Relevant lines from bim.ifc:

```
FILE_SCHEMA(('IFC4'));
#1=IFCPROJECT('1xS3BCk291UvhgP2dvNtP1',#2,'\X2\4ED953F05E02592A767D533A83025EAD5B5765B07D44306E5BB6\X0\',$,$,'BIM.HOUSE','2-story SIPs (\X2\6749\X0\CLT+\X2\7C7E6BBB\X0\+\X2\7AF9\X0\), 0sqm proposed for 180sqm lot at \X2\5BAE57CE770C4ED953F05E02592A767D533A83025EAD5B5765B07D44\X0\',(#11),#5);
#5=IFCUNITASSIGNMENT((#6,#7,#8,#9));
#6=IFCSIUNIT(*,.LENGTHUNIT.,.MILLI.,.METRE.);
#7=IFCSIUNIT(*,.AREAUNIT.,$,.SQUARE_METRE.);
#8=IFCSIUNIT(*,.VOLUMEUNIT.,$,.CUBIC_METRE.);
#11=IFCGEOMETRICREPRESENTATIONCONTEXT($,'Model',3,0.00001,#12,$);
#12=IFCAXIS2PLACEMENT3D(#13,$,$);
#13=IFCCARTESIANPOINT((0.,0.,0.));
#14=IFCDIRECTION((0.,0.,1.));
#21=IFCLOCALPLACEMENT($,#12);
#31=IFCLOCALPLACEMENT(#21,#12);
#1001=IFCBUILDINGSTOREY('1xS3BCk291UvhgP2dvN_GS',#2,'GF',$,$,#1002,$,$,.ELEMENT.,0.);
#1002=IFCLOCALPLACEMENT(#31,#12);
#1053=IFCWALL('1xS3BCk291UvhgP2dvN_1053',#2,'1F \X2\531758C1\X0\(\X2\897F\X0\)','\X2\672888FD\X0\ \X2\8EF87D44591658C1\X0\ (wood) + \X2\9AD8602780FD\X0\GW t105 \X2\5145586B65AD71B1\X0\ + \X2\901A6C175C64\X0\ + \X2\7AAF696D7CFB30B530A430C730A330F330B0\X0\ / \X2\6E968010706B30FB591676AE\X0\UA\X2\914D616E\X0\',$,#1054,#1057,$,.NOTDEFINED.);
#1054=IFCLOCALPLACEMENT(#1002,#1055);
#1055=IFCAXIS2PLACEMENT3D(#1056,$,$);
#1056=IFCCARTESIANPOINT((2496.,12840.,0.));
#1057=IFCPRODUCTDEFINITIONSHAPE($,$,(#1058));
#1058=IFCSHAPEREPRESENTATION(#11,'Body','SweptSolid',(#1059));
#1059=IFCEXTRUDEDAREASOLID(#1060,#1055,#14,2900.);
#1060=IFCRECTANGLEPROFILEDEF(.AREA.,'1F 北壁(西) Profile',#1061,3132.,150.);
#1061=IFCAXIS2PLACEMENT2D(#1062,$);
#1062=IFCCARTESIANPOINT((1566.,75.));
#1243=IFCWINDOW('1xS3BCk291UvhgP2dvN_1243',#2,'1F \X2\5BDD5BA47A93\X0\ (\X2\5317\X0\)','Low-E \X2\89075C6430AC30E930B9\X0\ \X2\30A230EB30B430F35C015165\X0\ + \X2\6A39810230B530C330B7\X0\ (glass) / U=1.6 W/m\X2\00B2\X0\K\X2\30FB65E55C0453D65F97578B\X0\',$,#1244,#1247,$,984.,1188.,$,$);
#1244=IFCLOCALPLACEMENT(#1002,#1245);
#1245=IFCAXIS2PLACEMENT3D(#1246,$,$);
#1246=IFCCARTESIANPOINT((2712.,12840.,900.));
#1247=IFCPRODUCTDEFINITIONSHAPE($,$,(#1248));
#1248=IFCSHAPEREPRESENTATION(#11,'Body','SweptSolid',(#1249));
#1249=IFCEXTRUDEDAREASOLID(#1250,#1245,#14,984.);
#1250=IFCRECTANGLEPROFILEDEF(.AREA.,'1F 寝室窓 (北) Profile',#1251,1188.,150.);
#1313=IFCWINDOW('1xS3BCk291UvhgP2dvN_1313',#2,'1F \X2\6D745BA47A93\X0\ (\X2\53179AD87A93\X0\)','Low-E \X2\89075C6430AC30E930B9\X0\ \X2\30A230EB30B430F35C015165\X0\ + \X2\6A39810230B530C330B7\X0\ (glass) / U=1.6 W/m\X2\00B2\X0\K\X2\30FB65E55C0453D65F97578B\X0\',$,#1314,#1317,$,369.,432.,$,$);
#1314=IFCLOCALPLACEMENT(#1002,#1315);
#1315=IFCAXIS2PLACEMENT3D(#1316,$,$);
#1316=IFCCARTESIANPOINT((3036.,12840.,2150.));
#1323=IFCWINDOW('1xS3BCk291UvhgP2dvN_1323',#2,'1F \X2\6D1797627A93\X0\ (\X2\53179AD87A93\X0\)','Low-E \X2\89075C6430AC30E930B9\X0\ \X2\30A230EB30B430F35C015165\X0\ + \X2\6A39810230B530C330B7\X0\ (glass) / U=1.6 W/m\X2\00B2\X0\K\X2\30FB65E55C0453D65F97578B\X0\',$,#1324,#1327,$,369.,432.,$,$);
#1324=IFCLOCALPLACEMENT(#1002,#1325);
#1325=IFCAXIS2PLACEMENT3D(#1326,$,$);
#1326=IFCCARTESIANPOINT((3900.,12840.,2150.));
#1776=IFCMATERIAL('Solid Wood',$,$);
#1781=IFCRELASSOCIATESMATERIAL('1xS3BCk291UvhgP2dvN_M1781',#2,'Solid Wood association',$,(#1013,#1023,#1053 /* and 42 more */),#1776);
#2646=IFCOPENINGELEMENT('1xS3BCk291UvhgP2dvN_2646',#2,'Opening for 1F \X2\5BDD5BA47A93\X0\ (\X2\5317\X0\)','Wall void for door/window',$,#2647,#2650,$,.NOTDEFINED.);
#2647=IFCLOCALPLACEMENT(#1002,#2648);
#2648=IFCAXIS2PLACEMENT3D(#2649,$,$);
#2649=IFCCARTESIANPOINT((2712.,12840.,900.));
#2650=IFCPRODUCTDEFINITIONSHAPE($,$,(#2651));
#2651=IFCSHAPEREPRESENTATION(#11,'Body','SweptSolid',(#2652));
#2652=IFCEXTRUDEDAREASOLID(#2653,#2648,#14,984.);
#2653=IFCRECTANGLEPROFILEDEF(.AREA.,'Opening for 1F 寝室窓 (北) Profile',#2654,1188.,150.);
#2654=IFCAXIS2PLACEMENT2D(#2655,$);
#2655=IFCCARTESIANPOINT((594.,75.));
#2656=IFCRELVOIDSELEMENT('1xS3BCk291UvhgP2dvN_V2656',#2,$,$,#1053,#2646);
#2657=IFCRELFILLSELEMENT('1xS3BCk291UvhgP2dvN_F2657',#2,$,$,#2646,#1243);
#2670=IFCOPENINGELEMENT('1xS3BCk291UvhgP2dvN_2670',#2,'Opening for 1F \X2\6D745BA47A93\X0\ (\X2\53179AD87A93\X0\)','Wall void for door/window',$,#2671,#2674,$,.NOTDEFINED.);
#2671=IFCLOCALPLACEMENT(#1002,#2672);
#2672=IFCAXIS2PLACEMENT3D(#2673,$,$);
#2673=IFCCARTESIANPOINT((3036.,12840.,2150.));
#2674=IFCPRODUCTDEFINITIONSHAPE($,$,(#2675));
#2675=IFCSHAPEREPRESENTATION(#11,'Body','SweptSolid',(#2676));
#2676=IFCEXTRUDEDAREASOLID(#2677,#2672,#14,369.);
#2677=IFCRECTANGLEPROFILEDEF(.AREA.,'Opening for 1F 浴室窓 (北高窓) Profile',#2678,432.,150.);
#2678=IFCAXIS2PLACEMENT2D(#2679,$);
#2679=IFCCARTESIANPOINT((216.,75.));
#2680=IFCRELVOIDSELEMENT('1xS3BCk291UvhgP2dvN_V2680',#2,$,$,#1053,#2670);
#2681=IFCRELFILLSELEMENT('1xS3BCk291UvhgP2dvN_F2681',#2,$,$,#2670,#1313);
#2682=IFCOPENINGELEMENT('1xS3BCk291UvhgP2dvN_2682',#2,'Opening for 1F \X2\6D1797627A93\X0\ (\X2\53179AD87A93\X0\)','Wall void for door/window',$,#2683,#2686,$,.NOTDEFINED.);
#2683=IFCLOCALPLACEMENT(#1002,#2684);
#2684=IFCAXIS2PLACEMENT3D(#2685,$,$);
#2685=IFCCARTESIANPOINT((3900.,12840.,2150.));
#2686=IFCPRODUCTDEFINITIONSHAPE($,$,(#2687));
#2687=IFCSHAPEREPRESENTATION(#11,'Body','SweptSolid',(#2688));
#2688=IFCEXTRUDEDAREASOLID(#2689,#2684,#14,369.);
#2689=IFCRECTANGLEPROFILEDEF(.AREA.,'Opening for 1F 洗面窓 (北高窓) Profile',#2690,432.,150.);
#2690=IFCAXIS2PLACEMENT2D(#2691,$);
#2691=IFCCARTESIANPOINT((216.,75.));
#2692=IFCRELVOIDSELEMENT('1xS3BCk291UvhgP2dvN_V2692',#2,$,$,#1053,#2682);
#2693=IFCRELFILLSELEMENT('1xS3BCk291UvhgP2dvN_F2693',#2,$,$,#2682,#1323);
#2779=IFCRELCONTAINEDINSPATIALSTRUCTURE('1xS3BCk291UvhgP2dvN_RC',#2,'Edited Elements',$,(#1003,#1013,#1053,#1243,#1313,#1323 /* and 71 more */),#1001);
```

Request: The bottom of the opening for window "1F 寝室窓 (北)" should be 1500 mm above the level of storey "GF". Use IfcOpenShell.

```python
import numpy as np
import ifcopenshell
import ifcopenshell.api.geometry
import ifcopenshell.geom
import ifcopenshell.util.element
import ifcopenshell.util.placement
import ifcopenshell.util.shape
import ifcopenshell.util.unit

model = ifcopenshell.open("bim.ifc")
unit_scale = ifcopenshell.util.unit.calculate_unit_scale(model)

window = model.by_id(1243)
opening = window.FillsVoids[0].RelatingOpeningElement
storey = ifcopenshell.util.element.get_container(window, ifc_class="IfcBuildingStorey")
level = ifcopenshell.util.placement.get_local_placement(storey.ObjectPlacement)[2, 3]

# The opening's origin need not be at the sill, so measure its lowest point.
shape = ifcopenshell.geom.create_shape(ifcopenshell.geom.settings(), opening)
bottom = ifcopenshell.util.shape.get_shape_bottom_elevation(shape, shape.geometry) / unit_scale
dz = level + 1.5 / unit_scale - bottom

shift = np.array([0.0, 0.0, dz])
# The window is not placed relative to its opening, so move both.
for product in (opening, window):
    matrix = ifcopenshell.util.placement.get_local_placement(product.ObjectPlacement)
    matrix[:3, 3] += shift
    ifcopenshell.api.geometry.edit_object_placement(model, product=product, matrix=matrix, is_si=False)

print(f"moved by {dz * unit_scale:+.3f} m")

model.write("bim_edited.ifc")
```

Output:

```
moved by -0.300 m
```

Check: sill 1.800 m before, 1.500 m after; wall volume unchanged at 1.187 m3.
